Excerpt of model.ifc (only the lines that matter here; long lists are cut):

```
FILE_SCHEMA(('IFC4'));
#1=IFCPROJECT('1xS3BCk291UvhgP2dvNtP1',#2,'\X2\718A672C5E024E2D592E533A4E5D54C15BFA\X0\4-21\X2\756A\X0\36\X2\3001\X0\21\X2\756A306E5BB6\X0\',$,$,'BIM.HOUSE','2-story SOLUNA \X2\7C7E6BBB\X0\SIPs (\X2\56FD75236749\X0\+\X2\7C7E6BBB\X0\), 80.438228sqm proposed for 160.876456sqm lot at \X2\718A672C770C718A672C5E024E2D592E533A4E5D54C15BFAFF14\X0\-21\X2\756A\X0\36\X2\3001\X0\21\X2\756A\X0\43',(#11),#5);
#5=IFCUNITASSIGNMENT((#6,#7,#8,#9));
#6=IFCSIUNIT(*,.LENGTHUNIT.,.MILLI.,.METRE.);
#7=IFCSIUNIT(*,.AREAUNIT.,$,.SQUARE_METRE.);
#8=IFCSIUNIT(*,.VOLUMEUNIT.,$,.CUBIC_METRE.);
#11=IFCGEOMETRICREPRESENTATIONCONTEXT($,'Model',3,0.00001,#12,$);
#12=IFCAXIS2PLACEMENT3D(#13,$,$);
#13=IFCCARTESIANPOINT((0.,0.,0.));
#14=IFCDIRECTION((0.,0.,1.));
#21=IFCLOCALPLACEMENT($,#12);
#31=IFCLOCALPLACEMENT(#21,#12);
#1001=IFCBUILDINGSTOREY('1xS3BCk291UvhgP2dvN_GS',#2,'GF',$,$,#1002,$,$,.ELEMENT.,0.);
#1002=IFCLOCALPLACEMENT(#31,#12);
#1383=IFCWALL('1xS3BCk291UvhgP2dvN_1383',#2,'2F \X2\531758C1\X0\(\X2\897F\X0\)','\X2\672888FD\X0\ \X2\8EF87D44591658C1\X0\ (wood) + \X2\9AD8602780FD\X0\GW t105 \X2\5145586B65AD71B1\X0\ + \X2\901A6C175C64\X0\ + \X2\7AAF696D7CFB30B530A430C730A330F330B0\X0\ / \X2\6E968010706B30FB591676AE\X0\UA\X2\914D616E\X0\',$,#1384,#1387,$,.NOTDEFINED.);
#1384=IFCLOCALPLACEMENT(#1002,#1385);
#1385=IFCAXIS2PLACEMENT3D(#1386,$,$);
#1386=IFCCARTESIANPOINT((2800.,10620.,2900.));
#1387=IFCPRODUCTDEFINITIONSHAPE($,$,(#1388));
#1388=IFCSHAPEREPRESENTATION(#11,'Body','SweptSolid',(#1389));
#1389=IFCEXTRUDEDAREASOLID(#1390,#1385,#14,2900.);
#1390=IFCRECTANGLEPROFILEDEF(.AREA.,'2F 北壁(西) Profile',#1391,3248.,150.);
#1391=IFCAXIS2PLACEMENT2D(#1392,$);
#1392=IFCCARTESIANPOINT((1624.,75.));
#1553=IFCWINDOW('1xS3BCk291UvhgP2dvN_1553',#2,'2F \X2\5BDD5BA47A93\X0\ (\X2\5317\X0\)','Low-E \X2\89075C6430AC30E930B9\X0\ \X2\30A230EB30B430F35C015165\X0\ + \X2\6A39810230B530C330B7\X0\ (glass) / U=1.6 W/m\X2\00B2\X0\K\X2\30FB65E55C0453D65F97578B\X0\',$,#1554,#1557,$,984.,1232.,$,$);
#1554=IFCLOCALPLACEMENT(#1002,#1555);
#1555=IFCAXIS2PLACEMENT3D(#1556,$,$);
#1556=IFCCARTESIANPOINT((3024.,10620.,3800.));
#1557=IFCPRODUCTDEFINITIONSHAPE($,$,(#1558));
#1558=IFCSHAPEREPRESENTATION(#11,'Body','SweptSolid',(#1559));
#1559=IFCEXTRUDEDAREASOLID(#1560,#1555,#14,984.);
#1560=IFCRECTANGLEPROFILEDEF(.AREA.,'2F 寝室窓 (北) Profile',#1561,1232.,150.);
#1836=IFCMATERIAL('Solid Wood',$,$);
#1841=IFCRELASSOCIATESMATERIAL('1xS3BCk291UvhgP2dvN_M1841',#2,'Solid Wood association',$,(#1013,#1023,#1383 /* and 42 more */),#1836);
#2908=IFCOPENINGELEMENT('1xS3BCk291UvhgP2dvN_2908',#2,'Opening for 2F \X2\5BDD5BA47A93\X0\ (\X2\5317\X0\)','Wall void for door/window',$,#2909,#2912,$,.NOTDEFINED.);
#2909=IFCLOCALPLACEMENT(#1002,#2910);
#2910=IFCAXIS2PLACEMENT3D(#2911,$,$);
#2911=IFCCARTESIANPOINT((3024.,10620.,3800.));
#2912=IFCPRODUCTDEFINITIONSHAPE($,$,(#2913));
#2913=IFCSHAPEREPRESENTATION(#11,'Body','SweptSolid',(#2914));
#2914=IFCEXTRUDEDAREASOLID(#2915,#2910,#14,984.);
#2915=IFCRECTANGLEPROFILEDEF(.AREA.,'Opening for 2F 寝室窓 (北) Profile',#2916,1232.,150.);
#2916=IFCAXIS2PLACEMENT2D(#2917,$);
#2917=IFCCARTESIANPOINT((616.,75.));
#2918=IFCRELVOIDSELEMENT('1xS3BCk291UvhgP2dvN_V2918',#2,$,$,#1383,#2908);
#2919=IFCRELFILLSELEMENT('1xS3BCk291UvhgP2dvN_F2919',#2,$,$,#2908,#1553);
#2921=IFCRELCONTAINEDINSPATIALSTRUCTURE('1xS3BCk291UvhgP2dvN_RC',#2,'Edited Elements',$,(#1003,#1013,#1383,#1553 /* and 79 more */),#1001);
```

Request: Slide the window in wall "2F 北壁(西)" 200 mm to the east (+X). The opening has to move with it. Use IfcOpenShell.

```python
import ifcopenshell
import ifcopenshell.api.geometry
import ifcopenshell.util.placement
import ifcopenshell.util.unit

model = ifcopenshell.open("model.ifc")
unit_scale = ifcopenshell.util.unit.calculate_unit_scale(model)

window = model.by_guid("1xS3BCk291UvhgP2dvN_1553")
opening = window.FillsVoids[0].RelatingOpeningElement
wall = opening.VoidsElements[0].RelatingBuildingElement

wall_matrix = ifcopenshell.util.placement.get_local_placement(wall.ObjectPlacement)
shift = wall_matrix[:3, 0] * 0.2 / unit_scale
before = ifcopenshell.util.placement.get_local_placement(window.ObjectPlacement)[:3, 3].copy()

# The window is not placed relative to its opening, so move both.
for product in (opening, window):
    matrix = ifcopenshell.util.placement.get_local_placement(product.ObjectPlacement)
    matrix[:3, 3] += shift
    ifcopenshell.api.geometry.edit_object_placement(model, product=product, matrix=matrix, is_si=False)

after = ifcopenshell.util.placement.get_local_placement(window.ObjectPlacement)[:3, 3]
print("window moved by", (after - before).round(3) + 0.0)

model.write("model_updated.ifc")
```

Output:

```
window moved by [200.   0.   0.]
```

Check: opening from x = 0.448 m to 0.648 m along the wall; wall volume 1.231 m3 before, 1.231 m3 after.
